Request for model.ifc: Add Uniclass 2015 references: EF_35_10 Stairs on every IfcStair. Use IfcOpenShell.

First a look at what the model holds.

```python
import ifcopenshell

model = ifcopenshell.open("model.ifc")
print(model.schema)
print("classifications:", [c.Name for c in model.by_type("IfcClassification")])
for ifc_class in ("IfcDoor", "IfcRoof", "IfcStair", "IfcWall", "IfcWindow"):
    print(ifc_class, len(model.by_type(ifc_class)))
```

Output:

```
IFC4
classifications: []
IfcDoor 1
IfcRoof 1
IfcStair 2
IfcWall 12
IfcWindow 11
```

```python
import ifcopenshell
import ifcopenshell.api.classification

model = ifcopenshell.open("model.ifc")

system = ifcopenshell.api.classification.add_classification(model, classification="Uniclass 2015")

codes = {
    "IfcStair": ("EF_35_10", "Stairs"),
}
for ifc_class, (code, name) in codes.items():
    products = model.by_type(ifc_class)
    ifcopenshell.api.classification.add_reference(
        model, products=products, classification=system, identification=code, name=name
    )
    print(code, len(products))

model.write("model_edited.ifc")
```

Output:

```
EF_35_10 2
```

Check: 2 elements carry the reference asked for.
